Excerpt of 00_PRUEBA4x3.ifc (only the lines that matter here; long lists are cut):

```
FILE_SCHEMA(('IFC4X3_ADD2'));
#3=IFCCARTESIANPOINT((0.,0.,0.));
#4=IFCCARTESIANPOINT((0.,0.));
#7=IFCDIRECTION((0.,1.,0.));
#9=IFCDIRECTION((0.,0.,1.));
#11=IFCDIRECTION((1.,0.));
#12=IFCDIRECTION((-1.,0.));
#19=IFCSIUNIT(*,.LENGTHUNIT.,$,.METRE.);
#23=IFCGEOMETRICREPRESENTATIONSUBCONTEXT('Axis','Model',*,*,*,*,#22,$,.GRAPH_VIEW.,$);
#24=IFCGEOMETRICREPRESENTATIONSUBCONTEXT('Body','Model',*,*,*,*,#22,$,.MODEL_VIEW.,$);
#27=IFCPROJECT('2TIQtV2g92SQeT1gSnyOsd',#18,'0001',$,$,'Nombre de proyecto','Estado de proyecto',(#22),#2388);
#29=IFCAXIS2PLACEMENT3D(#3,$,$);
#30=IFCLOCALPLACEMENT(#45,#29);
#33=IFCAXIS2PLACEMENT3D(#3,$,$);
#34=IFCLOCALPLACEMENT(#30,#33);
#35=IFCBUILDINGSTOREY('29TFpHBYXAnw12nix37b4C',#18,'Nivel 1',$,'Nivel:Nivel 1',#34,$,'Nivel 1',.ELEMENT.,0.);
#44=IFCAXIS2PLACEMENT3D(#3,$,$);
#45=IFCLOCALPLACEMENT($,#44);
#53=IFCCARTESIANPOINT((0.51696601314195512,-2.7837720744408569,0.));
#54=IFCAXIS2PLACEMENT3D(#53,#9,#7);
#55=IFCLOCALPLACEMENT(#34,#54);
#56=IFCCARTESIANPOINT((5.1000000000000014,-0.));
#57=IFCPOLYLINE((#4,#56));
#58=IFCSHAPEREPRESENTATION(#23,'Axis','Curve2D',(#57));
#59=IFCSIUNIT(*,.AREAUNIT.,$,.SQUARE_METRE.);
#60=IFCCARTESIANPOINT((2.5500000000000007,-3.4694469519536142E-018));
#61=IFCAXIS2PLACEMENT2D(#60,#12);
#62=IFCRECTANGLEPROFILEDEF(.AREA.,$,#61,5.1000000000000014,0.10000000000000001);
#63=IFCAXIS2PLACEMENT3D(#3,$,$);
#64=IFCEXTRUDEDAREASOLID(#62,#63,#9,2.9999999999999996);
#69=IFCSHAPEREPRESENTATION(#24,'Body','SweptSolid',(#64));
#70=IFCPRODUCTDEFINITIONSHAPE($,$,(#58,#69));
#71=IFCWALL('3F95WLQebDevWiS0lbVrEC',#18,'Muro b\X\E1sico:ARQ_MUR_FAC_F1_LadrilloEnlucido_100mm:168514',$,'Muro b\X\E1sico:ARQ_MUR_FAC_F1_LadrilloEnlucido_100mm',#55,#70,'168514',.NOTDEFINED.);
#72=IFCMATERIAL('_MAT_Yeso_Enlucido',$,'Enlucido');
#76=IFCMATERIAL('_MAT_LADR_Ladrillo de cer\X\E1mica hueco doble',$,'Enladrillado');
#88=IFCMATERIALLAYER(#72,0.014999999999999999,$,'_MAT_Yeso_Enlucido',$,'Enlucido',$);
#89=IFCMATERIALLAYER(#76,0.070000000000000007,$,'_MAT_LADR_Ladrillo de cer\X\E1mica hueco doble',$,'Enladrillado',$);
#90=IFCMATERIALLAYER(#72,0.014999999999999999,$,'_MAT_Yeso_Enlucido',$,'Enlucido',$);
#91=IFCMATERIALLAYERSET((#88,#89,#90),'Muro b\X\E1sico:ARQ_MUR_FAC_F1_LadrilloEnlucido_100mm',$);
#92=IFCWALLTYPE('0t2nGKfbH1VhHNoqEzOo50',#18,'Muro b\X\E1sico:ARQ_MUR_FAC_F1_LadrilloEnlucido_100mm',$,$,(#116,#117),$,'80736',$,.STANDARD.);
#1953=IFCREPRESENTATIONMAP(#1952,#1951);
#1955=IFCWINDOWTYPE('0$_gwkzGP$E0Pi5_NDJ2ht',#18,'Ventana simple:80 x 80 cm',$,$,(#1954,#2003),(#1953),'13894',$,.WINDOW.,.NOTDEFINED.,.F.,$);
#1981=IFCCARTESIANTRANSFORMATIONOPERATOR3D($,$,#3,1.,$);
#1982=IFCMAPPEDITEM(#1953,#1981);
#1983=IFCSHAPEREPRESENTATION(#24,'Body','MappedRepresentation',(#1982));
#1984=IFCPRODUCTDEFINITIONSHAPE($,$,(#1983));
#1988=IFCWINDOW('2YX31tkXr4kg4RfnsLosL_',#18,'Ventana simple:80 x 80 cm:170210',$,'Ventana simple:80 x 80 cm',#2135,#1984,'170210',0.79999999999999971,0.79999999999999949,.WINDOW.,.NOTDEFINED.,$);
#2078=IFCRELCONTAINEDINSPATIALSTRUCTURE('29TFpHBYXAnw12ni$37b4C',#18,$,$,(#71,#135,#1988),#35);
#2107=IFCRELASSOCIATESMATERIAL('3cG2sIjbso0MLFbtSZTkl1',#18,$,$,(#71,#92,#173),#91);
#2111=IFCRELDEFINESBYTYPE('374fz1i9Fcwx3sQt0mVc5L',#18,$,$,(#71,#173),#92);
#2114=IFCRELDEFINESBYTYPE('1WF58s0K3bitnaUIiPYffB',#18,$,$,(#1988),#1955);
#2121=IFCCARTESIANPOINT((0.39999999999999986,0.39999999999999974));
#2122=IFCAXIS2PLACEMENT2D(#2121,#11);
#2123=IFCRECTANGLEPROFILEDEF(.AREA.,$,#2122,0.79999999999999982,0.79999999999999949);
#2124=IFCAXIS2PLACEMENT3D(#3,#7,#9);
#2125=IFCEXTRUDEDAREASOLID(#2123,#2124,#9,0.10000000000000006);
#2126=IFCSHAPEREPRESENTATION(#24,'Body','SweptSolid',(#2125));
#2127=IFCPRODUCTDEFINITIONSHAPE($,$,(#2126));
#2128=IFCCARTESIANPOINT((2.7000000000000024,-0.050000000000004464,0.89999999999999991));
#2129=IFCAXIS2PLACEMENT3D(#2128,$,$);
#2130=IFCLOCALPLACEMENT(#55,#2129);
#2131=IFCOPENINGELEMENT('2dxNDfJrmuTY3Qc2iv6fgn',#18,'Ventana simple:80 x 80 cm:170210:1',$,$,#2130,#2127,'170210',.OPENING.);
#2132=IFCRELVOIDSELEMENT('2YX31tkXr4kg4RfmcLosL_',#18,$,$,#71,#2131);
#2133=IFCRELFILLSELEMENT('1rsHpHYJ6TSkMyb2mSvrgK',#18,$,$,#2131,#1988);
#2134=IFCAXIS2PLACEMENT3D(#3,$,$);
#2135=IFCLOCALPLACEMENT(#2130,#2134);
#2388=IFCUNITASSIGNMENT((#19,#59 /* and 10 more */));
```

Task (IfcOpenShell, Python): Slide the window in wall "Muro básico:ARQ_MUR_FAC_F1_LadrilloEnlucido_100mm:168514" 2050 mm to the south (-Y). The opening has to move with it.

```python
import ifcopenshell
import ifcopenshell.api.geometry
import ifcopenshell.util.placement
import ifcopenshell.util.unit

model = ifcopenshell.open("00_PRUEBA4x3.ifc")
unit_scale = ifcopenshell.util.unit.calculate_unit_scale(model)

window = model.by_id(1988)
opening = window.FillsVoids[0].RelatingOpeningElement
wall = opening.VoidsElements[0].RelatingBuildingElement

wall_matrix = ifcopenshell.util.placement.get_local_placement(wall.ObjectPlacement)
shift = wall_matrix[:3, 0] * -2.05 / unit_scale
before = ifcopenshell.util.placement.get_local_placement(window.ObjectPlacement)[:3, 3].copy()

# The window is placed relative to its opening, so it follows when the opening moves.
matrix = ifcopenshell.util.placement.get_local_placement(opening.ObjectPlacement)
matrix[:3, 3] += shift
ifcopenshell.api.geometry.edit_object_placement(
    model, product=opening, matrix=matrix, is_si=False, should_transform_children=True
)

after = ifcopenshell.util.placement.get_local_placement(window.ObjectPlacement)[:3, 3]
print("window moved by", (after - before).round(3) + 0.0)

model.write("00_PRUEBA4x3_edited.ifc")
```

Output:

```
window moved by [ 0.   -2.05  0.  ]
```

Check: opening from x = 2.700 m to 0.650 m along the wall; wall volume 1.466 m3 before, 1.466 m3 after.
